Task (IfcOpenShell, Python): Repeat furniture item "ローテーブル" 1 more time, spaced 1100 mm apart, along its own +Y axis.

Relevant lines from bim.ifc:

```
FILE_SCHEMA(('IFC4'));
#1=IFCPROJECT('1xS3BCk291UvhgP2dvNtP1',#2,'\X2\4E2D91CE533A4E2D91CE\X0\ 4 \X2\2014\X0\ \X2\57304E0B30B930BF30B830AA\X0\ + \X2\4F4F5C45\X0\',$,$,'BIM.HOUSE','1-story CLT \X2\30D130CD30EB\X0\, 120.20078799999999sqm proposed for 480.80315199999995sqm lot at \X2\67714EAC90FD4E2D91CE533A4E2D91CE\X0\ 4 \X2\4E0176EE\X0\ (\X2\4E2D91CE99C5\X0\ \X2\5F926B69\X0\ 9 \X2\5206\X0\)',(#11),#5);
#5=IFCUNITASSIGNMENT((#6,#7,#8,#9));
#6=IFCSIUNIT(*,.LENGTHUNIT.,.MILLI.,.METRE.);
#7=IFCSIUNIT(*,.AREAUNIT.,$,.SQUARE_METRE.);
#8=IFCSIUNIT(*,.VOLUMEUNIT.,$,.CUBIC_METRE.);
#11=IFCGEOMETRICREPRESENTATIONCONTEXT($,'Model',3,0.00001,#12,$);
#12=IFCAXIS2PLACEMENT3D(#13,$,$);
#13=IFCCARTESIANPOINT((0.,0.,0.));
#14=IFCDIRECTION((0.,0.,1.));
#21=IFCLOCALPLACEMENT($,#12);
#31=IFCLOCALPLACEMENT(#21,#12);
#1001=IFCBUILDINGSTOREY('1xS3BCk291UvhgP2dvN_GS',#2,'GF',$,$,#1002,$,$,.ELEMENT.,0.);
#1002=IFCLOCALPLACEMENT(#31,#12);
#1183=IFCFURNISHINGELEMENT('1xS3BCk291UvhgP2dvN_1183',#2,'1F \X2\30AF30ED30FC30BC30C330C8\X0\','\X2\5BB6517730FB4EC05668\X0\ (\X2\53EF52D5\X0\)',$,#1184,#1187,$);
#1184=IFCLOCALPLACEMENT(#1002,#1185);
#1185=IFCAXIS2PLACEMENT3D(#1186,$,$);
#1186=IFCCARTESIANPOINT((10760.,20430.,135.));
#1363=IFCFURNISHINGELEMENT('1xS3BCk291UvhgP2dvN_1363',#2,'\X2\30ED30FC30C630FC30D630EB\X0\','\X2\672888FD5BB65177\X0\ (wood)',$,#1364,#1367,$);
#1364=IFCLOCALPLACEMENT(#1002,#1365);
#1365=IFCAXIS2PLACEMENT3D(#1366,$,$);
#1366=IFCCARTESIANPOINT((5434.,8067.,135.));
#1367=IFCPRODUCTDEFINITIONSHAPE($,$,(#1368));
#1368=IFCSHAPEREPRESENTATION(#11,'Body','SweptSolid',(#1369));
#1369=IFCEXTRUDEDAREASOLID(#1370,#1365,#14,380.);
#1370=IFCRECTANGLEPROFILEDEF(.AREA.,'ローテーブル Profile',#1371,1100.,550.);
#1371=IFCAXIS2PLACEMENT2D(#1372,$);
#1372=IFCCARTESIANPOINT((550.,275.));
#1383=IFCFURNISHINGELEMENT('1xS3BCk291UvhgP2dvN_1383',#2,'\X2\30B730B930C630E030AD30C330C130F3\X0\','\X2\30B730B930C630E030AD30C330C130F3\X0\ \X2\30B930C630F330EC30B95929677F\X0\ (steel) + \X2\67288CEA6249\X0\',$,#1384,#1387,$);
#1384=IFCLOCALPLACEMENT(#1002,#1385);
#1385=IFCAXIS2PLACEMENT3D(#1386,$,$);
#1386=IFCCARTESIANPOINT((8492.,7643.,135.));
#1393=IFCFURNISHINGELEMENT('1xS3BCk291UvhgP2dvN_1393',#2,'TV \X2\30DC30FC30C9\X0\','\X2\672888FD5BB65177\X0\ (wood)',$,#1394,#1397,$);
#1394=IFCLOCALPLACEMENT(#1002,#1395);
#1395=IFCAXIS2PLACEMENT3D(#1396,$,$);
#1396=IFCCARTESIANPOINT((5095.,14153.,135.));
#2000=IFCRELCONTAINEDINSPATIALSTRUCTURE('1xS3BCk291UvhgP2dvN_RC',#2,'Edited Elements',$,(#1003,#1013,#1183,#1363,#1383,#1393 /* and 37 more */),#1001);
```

```python
import ifcopenshell
import ifcopenshell.api.geometry
import ifcopenshell.api.root
import ifcopenshell.util.element
import ifcopenshell.util.placement
import ifcopenshell.util.unit

model = ifcopenshell.open("bim.ifc")
unit_scale = ifcopenshell.util.unit.calculate_unit_scale(model)


def reuse_history(source, copy):
    """copy_class also copies each property set's owner history, people and application; keep the originals."""
    for rel in copy.IsDefinedBy:
        if rel.is_a("IfcRelDefinesByProperties") and (history := rel.RelatingPropertyDefinition.OwnerHistory):
            rel.RelatingPropertyDefinition.OwnerHistory = source.OwnerHistory
            ifcopenshell.util.element.remove_deep2(model, history)


source = model.by_id(1363)
base = ifcopenshell.util.placement.get_local_placement(source.ObjectPlacement)
step = base[:3, 1] * 1.1 / unit_scale

for i in range(1, 2):
    copy = ifcopenshell.api.root.copy_class(model, product=source)
    copy.Representation = ifcopenshell.util.element.copy_deep(
        model, source.Representation, exclude=["IfcGeometricRepresentationContext", "IfcRepresentationMap"]
    )
    reuse_history(source, copy)
    matrix = base.copy()
    matrix[:3, 3] += i * step
    print("added at", matrix[:3, 3].round(3) + 0.0)
    ifcopenshell.api.geometry.edit_object_placement(model, product=copy, matrix=matrix, is_si=False)

model.write("bim_rev.ifc")
```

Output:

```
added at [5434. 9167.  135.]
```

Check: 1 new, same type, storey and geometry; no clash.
